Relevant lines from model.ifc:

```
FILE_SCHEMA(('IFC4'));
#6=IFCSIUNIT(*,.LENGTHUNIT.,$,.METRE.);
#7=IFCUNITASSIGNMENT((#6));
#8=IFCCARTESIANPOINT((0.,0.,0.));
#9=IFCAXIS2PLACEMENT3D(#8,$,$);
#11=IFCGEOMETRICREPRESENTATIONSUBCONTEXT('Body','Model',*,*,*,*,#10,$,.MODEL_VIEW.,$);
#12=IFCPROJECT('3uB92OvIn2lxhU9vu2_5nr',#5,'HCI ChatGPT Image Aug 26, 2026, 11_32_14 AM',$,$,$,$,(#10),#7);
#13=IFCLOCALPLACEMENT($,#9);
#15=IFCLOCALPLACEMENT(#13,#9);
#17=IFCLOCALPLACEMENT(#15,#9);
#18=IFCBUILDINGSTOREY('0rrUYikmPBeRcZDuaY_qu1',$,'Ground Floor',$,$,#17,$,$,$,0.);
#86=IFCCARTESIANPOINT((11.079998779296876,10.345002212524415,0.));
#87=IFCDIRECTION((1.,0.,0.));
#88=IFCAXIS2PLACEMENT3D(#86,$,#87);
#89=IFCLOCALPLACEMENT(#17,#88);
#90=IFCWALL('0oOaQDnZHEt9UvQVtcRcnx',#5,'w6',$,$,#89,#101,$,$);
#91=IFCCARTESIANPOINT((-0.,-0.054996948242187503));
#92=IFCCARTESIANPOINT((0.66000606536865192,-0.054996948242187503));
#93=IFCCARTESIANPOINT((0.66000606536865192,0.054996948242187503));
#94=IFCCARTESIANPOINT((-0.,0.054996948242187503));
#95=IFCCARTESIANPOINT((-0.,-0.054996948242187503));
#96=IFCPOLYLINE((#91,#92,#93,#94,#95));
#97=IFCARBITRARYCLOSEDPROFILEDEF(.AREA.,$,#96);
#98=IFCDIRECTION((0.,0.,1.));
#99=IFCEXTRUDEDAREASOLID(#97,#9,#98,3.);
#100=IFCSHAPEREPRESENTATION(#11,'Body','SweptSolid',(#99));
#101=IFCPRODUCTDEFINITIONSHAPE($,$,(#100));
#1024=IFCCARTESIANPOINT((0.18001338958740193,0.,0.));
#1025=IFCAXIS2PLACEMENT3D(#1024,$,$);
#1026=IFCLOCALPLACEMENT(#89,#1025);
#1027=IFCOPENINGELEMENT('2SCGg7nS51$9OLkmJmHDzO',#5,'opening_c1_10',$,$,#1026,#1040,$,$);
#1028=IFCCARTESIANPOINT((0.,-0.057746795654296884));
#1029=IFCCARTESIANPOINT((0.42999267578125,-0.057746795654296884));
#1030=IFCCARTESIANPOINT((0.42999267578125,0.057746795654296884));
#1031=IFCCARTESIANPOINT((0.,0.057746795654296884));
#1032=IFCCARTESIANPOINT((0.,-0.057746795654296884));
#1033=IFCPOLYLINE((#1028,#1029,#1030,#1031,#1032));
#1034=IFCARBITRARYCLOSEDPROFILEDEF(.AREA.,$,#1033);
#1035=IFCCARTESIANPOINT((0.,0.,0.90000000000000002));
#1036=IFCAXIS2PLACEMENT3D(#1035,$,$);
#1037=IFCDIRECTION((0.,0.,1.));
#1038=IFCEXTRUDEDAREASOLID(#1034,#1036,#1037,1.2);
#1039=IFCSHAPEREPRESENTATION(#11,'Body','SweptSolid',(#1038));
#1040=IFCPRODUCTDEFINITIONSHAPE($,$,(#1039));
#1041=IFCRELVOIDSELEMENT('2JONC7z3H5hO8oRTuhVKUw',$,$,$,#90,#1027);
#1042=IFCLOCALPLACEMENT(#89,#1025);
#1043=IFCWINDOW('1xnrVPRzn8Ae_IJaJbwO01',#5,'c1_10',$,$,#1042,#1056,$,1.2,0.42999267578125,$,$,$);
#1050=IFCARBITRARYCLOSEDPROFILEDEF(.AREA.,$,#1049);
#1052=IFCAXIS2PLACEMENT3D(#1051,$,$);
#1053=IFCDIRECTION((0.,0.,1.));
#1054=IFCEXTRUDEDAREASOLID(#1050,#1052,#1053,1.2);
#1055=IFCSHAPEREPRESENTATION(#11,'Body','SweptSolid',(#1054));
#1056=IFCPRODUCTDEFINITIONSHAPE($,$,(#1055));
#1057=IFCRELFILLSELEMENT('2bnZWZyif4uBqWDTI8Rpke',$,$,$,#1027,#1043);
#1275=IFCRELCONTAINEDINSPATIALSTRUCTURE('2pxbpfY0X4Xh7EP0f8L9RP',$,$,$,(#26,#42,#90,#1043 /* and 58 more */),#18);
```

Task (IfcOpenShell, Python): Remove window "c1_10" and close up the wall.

```python
import ifcopenshell
import ifcopenshell.api.feature
import ifcopenshell.api.root
import ifcopenshell.geom
import ifcopenshell.util.shape

model = ifcopenshell.open("model.ifc")
settings = ifcopenshell.geom.settings()


def volume(element):
    """Net volume in cubic metres, openings subtracted."""
    shape = ifcopenshell.geom.create_shape(settings, element)
    return ifcopenshell.util.shape.get_volume(shape.geometry)


window = model.by_guid("1xnrVPRzn8Ae_IJaJbwO01")
opening = window.FillsVoids[0].RelatingOpeningElement
wall = opening.VoidsElements[0].RelatingBuildingElement
before = volume(wall)

ifcopenshell.api.root.remove_product(model, product=window)
ifcopenshell.api.feature.remove_feature(model, feature=opening)

after = volume(wall)

print(f"wall volume {before:.3f} -> {after:.3f} m3")

model.write("model-out.ifc")
```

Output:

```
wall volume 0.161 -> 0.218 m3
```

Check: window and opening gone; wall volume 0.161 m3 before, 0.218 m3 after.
